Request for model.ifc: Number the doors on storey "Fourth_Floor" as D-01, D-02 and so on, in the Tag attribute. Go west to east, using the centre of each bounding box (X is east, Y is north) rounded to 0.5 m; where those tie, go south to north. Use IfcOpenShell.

First a look at what the model holds.

```python
import ifcopenshell
import ifcopenshell.util.element
import ifcopenshell.util.placement

model = ifcopenshell.open("model.ifc")
print(model.schema)
storey = next(s for s in model.by_type("IfcBuildingStorey") if s.Name == "Fourth_Floor")
doors = [e for e in ifcopenshell.util.element.get_decomposition(storey) if e.is_a("IfcDoor")]
for e in sorted(doors, key=lambda e: e.id()):
    origin = ifcopenshell.util.placement.get_local_placement(e.ObjectPlacement)[:3, 3]
    print(e.id(), e.Tag, e.Name, origin.round(2) + 0.0, sep=" | ")
```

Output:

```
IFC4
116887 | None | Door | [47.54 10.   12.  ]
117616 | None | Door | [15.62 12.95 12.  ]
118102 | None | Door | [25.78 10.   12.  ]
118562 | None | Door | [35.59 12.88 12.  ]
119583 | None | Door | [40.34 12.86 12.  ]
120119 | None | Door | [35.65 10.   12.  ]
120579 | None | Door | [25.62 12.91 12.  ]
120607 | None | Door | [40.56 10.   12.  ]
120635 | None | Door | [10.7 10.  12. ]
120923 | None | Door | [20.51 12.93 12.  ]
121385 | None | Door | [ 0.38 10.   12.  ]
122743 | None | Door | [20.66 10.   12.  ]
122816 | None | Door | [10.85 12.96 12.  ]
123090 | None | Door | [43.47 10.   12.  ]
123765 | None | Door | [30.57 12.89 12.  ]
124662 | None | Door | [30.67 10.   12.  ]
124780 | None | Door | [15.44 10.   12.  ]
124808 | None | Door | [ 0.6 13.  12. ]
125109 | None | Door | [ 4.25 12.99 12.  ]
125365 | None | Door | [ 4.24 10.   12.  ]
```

```python
import ifcopenshell
import ifcopenshell.geom
import ifcopenshell.util.element
import ifcopenshell.util.shape

model = ifcopenshell.open("model.ifc")
settings = ifcopenshell.geom.settings()
settings.set("use-world-coords", True)


def centre(element):
    shape = ifcopenshell.geom.create_shape(settings, element)
    return ifcopenshell.util.shape.get_bbox_centroid(shape.geometry)


storey = next(s for s in model.by_type("IfcBuildingStorey") if s.Name == "Fourth_Floor")
doors = [e for e in ifcopenshell.util.element.get_decomposition(storey) if e.is_a("IfcDoor")]

# Insertion points can sit at a corner or the storey origin, so sort by the geometry (in metres).
centres = {e: centre(e) for e in doors}
doors.sort(key=lambda e: (round(centres[e][0] / 0.5), centres[e][1]))

for i, e in enumerate(doors, start=1):
    number = f"D-{i:02d}"
    e.Tag = number
    print(e.id(), number)

model.write("model_v2.ifc")
```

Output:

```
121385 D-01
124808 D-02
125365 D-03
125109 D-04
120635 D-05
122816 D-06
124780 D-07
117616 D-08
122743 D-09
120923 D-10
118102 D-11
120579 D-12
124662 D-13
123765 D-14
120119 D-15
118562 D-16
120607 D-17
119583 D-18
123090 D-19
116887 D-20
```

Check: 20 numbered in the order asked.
